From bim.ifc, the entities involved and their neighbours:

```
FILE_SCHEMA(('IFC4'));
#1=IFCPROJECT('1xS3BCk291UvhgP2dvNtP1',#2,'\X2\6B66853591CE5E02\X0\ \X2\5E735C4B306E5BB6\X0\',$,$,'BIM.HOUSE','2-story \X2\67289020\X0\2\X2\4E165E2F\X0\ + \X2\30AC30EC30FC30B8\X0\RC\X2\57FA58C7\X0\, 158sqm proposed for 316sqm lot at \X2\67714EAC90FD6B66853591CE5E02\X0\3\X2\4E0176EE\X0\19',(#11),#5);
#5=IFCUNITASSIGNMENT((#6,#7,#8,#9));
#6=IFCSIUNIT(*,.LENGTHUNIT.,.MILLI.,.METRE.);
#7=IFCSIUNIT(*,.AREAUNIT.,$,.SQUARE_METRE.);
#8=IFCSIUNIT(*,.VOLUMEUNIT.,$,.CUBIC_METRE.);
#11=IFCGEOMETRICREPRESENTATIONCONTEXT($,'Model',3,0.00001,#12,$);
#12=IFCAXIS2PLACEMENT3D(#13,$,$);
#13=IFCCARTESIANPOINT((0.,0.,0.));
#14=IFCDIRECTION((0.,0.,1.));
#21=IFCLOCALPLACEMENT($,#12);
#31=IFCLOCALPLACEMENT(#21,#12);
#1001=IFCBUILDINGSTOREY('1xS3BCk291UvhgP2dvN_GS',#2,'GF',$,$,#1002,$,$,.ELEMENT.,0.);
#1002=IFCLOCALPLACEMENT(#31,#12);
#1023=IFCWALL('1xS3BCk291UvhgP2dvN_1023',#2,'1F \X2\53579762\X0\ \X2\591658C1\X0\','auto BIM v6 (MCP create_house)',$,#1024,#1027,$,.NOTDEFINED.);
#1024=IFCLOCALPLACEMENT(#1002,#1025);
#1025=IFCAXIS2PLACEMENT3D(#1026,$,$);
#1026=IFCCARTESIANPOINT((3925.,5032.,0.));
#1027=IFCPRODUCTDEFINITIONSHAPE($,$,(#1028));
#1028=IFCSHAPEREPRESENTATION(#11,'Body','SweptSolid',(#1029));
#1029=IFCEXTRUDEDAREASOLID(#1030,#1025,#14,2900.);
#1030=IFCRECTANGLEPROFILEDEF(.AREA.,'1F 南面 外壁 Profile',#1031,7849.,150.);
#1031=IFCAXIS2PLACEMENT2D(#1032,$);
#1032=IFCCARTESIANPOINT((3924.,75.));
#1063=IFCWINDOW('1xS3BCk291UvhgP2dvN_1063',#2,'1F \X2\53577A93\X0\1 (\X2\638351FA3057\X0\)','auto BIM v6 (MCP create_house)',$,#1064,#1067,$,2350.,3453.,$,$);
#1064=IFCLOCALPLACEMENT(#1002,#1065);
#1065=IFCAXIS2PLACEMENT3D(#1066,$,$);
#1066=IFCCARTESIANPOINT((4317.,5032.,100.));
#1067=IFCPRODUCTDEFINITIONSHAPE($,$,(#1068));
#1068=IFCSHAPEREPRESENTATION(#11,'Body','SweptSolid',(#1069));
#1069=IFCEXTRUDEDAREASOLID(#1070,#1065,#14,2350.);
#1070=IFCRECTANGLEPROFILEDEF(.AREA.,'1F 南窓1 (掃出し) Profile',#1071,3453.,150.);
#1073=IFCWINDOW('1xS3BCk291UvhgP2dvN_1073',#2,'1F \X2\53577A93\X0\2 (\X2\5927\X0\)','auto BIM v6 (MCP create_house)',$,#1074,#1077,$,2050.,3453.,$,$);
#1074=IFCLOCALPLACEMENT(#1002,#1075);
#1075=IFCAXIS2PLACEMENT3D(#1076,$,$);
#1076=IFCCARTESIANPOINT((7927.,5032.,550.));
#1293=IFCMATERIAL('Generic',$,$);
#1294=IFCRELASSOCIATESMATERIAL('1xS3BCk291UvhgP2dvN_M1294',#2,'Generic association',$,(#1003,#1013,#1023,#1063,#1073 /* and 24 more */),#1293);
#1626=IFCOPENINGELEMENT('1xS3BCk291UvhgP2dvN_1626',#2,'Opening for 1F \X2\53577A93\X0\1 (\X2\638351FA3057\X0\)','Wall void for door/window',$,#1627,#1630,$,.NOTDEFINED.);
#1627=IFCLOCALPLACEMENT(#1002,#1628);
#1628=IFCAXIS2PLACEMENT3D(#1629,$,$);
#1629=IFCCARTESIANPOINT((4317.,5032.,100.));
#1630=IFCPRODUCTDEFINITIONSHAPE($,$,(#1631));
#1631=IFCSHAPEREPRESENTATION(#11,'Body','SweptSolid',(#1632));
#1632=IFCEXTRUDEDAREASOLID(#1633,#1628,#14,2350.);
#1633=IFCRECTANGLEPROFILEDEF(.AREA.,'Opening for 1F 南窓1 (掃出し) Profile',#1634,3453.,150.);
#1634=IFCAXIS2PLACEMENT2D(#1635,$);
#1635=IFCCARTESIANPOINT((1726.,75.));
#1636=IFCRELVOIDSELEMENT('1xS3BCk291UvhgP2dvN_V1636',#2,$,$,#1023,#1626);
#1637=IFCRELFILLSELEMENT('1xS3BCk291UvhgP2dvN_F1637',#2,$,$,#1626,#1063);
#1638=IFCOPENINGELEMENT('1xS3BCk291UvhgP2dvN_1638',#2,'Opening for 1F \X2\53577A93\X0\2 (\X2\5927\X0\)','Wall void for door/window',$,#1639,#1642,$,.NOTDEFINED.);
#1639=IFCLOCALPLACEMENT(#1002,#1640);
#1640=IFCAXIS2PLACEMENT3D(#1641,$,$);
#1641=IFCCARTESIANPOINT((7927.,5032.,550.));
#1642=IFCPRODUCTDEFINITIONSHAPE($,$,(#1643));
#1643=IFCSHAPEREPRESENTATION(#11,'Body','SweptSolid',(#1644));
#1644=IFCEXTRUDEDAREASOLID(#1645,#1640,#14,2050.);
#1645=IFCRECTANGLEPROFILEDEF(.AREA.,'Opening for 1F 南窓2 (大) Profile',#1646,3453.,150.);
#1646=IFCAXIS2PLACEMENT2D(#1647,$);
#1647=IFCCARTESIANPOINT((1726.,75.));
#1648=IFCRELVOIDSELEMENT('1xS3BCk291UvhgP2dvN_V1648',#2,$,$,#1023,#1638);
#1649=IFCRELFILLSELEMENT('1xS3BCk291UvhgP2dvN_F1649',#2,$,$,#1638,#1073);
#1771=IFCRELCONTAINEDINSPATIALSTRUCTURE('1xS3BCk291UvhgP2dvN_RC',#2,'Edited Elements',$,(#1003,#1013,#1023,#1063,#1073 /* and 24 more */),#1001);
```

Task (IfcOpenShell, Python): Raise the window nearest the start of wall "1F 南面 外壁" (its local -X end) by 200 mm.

```python
import numpy as np
import ifcopenshell
import ifcopenshell.api.geometry
import ifcopenshell.util.placement
import ifcopenshell.util.unit

model = ifcopenshell.open("bim.ifc")
unit_scale = ifcopenshell.util.unit.calculate_unit_scale(model)

window = model.by_guid("1xS3BCk291UvhgP2dvN_1063")
opening = window.FillsVoids[0].RelatingOpeningElement
dz = 0.2 / unit_scale

shift = np.array([0.0, 0.0, dz])
# The window is not placed relative to its opening, so move both.
for product in (opening, window):
    matrix = ifcopenshell.util.placement.get_local_placement(product.ObjectPlacement)
    matrix[:3, 3] += shift
    ifcopenshell.api.geometry.edit_object_placement(model, product=product, matrix=matrix, is_si=False)

print(f"moved by {dz * unit_scale:+.3f} m")

model.write("bim_rev.ifc")
```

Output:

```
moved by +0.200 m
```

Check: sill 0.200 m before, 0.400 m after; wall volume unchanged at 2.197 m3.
